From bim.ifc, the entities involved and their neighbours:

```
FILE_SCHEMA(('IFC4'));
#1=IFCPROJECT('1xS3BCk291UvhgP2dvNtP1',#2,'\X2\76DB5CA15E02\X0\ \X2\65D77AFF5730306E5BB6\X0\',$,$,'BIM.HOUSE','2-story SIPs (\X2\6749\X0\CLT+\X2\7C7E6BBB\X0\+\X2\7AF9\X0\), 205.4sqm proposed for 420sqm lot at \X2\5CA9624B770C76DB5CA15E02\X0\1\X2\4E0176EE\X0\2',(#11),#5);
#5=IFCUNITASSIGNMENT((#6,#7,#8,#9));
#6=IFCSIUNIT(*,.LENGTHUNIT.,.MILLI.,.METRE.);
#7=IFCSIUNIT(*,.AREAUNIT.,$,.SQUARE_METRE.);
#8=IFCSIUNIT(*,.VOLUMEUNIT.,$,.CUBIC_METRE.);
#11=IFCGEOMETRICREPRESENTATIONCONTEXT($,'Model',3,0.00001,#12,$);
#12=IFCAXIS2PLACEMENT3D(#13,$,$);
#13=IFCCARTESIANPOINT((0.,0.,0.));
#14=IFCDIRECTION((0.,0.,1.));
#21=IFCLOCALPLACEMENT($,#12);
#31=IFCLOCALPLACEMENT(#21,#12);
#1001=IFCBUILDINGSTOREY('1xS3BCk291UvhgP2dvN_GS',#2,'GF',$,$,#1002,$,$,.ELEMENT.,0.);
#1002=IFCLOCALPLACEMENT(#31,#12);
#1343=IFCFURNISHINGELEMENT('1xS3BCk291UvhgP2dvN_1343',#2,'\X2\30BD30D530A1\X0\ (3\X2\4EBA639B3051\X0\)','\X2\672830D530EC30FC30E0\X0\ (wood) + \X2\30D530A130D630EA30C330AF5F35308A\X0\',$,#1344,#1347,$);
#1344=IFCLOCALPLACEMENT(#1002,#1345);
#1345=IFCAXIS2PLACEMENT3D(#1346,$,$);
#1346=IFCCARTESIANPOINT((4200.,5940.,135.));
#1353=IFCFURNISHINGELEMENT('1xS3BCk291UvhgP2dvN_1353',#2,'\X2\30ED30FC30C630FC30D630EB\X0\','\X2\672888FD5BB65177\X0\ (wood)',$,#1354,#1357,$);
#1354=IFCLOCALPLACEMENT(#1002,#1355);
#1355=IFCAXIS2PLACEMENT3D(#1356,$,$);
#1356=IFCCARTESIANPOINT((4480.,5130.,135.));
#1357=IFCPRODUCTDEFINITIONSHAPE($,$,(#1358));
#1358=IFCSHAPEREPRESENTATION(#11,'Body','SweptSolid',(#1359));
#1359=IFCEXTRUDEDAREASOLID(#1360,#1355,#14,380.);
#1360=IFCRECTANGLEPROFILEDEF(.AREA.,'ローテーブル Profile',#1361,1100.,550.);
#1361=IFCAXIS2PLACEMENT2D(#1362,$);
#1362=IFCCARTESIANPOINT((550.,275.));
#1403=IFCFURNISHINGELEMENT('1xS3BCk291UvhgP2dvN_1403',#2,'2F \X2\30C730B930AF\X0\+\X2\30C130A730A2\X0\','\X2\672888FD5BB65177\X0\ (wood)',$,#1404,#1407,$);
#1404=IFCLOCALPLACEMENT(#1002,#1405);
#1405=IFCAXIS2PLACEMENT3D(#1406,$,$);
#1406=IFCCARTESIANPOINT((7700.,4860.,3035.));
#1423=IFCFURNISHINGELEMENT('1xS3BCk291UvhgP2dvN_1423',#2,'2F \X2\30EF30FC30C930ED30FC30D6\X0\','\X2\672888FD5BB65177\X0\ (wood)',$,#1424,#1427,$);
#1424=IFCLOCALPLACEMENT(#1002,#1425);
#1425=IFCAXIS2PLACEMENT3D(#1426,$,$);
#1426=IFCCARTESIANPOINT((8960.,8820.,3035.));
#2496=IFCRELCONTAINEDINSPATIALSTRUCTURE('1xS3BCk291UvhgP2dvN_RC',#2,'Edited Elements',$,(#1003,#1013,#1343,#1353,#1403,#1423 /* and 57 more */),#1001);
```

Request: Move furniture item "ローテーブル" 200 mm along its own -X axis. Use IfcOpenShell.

```python
import ifcopenshell
import ifcopenshell.api.geometry
import ifcopenshell.util.placement

model = ifcopenshell.open("bim.ifc")

item = model.by_id(1353)
matrix = ifcopenshell.util.placement.get_local_placement(item.ObjectPlacement)
matrix[:3, 3] -= matrix[:3, 0] * 200.0
ifcopenshell.api.geometry.edit_object_placement(model, product=item, matrix=matrix, is_si=False)

print(ifcopenshell.util.placement.get_local_placement(item.ObjectPlacement).round(3) + 0.0)

model.write("bim_updated.ifc")
```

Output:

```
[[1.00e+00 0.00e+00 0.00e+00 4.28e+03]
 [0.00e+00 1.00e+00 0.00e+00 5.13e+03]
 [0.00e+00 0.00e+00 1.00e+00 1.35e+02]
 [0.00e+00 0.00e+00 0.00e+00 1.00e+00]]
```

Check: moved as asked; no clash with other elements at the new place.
